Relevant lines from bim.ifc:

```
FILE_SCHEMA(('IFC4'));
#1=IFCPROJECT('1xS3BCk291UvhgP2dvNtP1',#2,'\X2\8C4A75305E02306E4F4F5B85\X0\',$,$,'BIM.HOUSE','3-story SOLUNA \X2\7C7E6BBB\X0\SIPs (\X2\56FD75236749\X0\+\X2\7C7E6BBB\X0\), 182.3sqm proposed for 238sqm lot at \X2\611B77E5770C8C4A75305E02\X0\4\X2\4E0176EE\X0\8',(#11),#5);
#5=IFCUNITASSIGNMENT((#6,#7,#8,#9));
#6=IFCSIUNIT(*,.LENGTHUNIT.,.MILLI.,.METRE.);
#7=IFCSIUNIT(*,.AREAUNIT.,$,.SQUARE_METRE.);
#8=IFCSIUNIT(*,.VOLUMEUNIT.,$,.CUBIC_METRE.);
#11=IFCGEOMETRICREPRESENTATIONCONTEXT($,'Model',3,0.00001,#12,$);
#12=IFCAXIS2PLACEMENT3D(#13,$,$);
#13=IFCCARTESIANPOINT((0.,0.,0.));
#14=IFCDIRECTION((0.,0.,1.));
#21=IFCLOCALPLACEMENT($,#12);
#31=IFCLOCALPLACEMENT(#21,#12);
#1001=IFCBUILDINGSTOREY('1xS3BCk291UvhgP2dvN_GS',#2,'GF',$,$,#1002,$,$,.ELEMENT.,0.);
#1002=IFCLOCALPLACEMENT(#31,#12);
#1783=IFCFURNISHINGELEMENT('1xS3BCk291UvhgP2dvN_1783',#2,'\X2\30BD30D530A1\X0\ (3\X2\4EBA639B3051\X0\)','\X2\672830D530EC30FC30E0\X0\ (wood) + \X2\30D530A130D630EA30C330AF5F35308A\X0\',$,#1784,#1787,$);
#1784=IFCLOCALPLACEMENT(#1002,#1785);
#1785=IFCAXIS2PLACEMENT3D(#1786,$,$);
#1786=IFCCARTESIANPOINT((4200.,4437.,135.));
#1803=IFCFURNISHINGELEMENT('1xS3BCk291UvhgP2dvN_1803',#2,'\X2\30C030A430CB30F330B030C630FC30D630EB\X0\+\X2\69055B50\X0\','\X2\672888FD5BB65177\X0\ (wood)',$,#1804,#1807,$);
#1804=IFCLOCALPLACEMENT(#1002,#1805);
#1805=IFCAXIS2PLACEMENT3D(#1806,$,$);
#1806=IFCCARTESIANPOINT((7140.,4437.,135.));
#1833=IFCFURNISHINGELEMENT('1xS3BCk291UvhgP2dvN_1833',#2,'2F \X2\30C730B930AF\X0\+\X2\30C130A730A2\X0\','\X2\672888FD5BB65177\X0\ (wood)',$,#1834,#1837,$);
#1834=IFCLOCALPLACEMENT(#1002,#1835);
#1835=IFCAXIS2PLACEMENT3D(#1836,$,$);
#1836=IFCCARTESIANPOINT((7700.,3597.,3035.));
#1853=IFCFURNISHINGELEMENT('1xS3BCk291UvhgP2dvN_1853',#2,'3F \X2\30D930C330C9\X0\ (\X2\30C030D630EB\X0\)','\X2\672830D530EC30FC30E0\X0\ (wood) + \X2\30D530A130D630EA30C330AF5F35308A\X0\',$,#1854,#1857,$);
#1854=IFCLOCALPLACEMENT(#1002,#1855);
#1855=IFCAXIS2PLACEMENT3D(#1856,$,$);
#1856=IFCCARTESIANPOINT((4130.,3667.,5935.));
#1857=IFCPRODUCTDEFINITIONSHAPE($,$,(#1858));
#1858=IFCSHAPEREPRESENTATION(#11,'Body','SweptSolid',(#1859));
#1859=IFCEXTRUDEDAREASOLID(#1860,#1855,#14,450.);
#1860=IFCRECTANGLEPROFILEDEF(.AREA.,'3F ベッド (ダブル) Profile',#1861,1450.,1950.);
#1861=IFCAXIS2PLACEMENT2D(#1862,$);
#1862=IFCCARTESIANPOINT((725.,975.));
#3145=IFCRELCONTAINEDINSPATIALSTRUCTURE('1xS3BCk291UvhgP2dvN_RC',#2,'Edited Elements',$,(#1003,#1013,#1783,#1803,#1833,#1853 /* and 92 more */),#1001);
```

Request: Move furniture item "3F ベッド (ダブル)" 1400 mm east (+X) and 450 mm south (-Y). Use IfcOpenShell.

```python
import ifcopenshell
import ifcopenshell.api.geometry
import ifcopenshell.util.placement
import ifcopenshell.util.unit

model = ifcopenshell.open("bim.ifc")
unit_scale = ifcopenshell.util.unit.calculate_unit_scale(model)

item = model.by_guid("1xS3BCk291UvhgP2dvN_1853")
matrix = ifcopenshell.util.placement.get_local_placement(item.ObjectPlacement)
matrix[0, 3] += 1.4 / unit_scale
matrix[1, 3] -= 0.45 / unit_scale
ifcopenshell.api.geometry.edit_object_placement(model, product=item, matrix=matrix, is_si=False)

print(ifcopenshell.util.placement.get_local_placement(item.ObjectPlacement).round(3) + 0.0)

model.write("bim_updated.ifc")
```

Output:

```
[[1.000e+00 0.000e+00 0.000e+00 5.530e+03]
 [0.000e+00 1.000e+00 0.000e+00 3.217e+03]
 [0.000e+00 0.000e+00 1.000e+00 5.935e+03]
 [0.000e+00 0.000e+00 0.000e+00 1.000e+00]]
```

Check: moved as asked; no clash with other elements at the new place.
